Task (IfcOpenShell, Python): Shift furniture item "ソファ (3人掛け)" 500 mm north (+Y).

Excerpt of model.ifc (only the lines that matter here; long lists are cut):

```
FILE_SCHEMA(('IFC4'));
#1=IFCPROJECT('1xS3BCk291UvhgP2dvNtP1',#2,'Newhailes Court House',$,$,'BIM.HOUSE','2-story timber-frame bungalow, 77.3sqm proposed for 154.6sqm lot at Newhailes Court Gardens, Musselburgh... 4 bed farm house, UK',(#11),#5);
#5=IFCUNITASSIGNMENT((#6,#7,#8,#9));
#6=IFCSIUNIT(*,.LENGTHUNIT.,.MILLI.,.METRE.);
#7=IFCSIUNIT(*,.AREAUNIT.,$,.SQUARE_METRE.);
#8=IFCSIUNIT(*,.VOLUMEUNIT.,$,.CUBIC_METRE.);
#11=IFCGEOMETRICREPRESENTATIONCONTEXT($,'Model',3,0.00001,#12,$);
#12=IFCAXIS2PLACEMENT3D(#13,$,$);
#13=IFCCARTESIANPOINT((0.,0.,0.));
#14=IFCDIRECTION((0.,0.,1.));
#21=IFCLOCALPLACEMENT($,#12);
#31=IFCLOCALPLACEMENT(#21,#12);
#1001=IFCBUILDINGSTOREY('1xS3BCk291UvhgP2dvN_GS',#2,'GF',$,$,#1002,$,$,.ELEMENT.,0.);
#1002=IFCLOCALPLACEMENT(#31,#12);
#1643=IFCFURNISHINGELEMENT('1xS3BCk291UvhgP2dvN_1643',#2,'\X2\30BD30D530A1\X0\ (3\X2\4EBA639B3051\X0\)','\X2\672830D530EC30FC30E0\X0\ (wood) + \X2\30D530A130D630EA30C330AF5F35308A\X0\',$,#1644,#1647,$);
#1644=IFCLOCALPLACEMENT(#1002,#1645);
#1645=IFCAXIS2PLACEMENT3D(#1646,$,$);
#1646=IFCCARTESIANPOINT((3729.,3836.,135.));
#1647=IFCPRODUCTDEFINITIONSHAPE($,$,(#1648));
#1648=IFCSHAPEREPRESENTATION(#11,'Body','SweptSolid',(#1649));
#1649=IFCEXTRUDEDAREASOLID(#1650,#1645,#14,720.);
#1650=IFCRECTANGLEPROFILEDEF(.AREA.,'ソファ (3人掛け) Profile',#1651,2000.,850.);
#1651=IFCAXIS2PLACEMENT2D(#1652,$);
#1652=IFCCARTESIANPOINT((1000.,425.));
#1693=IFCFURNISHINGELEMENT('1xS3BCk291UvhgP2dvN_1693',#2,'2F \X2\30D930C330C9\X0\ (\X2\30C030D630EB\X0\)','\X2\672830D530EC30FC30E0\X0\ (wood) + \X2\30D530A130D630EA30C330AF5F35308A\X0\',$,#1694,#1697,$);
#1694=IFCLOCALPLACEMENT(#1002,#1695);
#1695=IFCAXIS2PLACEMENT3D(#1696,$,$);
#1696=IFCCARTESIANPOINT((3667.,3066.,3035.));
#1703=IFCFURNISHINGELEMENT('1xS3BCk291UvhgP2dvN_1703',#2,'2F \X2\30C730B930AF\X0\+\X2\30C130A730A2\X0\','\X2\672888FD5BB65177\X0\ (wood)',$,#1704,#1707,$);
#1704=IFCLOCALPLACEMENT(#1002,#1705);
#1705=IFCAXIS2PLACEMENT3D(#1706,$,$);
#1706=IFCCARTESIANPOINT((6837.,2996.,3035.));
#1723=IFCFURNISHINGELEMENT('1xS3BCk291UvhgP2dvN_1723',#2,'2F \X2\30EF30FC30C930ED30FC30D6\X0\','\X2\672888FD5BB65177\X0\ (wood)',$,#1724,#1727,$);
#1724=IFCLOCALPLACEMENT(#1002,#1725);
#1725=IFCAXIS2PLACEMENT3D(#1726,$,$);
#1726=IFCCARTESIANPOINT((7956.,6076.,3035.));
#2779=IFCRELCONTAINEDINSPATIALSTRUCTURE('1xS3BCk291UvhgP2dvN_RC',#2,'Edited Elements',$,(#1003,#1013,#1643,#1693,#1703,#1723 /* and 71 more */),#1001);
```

```python
import ifcopenshell
import ifcopenshell.api.geometry
import ifcopenshell.util.placement
import ifcopenshell.util.unit

model = ifcopenshell.open("model.ifc")
unit_scale = ifcopenshell.util.unit.calculate_unit_scale(model)

item = model.by_guid("1xS3BCk291UvhgP2dvN_1643")
matrix = ifcopenshell.util.placement.get_local_placement(item.ObjectPlacement)
matrix[1, 3] += 0.5 / unit_scale
ifcopenshell.api.geometry.edit_object_placement(model, product=item, matrix=matrix, is_si=False)

print(ifcopenshell.util.placement.get_local_placement(item.ObjectPlacement).round(3) + 0.0)

model.write("model_updated.ifc")
```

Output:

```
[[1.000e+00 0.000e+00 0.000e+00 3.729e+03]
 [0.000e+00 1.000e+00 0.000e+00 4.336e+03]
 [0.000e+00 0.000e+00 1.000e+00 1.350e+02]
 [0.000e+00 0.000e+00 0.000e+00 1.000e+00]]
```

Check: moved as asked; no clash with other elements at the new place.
